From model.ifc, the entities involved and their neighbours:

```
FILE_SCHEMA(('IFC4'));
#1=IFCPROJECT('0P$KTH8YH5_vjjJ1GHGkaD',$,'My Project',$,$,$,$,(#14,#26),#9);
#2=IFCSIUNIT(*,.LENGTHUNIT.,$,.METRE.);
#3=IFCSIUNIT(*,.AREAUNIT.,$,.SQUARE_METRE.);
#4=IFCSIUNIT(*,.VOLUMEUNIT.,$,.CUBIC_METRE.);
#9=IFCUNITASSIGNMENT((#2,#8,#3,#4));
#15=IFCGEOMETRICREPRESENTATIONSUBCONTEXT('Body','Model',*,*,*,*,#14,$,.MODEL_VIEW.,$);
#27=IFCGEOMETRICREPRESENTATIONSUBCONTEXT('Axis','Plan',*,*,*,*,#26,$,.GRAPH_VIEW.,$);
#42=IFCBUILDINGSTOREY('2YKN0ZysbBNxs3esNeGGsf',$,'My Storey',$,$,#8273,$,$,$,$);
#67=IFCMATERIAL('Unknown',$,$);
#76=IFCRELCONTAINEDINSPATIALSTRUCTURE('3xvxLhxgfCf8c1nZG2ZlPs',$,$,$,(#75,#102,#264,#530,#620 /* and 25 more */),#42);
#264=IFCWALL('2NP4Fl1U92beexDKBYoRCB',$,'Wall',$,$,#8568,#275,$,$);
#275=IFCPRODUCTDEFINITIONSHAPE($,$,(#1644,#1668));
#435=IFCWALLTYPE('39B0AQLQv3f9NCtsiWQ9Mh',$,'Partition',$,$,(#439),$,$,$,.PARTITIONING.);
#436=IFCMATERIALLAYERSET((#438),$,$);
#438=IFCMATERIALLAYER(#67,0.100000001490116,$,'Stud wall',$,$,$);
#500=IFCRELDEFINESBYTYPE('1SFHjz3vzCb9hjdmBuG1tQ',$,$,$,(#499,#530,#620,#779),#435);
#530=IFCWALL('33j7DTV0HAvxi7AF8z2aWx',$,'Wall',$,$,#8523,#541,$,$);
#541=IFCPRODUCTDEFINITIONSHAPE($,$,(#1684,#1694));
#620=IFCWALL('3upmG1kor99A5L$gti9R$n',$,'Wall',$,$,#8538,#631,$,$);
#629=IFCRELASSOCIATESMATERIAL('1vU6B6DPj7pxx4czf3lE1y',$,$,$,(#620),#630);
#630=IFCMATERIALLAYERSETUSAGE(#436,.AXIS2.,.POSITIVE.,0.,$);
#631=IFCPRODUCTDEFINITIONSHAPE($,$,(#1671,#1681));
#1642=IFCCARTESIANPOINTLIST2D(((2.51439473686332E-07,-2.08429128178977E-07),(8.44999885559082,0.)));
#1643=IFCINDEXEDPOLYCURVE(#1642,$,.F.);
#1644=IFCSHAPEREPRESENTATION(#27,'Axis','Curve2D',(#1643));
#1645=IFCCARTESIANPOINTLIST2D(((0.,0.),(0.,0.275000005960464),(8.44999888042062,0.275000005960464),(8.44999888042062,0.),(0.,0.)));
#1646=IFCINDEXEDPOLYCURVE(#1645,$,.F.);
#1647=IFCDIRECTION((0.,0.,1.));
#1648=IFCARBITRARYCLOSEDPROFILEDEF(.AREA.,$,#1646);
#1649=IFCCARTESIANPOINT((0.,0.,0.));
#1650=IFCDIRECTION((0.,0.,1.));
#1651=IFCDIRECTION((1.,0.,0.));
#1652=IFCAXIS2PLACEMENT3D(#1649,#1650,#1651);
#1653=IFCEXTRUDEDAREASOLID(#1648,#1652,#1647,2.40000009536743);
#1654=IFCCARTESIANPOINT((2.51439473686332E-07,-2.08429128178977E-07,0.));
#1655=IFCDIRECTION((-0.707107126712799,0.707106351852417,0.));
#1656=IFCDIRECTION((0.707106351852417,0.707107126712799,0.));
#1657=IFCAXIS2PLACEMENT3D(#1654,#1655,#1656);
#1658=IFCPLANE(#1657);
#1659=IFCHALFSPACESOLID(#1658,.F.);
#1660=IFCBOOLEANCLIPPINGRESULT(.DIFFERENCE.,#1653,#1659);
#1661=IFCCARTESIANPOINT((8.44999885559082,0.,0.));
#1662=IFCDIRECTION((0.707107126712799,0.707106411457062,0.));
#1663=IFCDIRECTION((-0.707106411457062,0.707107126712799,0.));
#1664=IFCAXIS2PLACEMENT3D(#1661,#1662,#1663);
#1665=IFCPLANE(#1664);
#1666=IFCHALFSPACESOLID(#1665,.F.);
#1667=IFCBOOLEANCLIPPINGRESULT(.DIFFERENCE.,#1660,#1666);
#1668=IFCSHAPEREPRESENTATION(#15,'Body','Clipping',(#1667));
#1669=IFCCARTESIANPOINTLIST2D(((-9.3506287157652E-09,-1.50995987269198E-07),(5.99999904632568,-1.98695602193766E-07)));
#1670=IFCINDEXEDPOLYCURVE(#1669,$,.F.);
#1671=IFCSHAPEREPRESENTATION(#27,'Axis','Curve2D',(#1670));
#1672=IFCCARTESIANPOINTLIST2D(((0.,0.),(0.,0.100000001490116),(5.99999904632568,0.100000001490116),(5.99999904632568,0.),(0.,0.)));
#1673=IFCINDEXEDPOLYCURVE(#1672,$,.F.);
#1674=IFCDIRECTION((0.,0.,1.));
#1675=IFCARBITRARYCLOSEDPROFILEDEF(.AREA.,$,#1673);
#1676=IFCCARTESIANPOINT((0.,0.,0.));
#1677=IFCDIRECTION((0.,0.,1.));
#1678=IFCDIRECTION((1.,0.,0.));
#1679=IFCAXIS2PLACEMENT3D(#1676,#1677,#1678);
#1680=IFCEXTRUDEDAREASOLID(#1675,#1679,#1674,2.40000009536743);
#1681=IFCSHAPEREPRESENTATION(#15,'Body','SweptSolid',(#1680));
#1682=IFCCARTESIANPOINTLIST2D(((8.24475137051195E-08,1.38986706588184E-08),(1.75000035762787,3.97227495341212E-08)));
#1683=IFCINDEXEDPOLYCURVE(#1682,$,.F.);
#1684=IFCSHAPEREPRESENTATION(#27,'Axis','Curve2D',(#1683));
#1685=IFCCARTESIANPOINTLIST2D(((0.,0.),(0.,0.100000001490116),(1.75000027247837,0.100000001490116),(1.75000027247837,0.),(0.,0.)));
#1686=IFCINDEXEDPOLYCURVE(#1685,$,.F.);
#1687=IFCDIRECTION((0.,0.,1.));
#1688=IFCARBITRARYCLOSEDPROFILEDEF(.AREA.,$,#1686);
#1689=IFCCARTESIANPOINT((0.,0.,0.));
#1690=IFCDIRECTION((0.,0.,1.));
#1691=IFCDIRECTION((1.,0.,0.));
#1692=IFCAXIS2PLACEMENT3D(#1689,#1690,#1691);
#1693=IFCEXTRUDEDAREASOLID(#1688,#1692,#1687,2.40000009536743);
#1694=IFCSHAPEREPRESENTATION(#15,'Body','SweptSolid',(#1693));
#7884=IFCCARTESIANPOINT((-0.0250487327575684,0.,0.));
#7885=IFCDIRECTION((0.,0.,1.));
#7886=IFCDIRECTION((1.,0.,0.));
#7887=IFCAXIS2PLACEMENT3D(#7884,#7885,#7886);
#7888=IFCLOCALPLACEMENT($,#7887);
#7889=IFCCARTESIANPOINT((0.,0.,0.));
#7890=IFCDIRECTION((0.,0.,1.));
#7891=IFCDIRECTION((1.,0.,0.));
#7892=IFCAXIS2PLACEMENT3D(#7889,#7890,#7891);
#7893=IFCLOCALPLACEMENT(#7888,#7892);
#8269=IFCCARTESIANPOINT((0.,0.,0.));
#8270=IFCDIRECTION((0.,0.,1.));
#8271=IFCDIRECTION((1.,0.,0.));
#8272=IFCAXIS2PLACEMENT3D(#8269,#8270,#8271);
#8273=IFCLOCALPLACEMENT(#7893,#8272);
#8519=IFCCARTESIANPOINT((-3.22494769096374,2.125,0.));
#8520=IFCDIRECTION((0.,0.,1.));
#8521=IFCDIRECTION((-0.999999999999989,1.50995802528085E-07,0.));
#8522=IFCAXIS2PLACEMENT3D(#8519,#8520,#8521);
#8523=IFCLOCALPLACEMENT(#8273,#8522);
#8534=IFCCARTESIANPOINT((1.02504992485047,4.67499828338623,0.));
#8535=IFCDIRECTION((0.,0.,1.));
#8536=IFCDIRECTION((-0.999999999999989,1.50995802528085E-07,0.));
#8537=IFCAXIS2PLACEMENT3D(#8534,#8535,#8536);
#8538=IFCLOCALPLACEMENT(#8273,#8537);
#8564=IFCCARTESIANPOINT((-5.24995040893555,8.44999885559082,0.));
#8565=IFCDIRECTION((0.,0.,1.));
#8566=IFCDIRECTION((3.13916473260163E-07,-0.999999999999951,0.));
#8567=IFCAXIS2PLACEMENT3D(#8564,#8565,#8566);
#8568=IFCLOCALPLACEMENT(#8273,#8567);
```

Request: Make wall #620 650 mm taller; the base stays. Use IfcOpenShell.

```python
import ifcopenshell
import ifcopenshell.geom
import ifcopenshell.util.representation
import ifcopenshell.util.shape

model = ifcopenshell.open("model.ifc")
settings = ifcopenshell.geom.settings()


def volume(element):
    """Net volume in cubic metres, openings subtracted."""
    shape = ifcopenshell.geom.create_shape(settings, element)
    return ifcopenshell.util.shape.get_volume(shape.geometry)


wall = model.by_guid("3upmG1kor99A5L$gti9R$n")
before = volume(wall)

body = ifcopenshell.util.representation.get_representation(wall, "Model", "Body")
solid = body.Items[0]
old_height = solid.Depth
solid.Depth += 0.65
after = volume(wall)

print(f"height {old_height:g} -> {solid.Depth:g}, volume {before:.3f} -> {after:.3f} m3")

model.write("model_edited.ifc")
```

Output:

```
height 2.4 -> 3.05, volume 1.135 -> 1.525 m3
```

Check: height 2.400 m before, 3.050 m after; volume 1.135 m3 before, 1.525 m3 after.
